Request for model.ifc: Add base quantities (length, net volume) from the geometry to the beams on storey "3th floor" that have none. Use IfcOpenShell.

First a look at what the model holds.

```python
import ifcopenshell
import ifcopenshell.util.element
import ifcopenshell.util.unit

model = ifcopenshell.open("model.ifc")
print(model.schema)
for unit_type in ("LENGTHUNIT", "AREAUNIT", "VOLUMEUNIT"):
    print(unit_type, ifcopenshell.util.unit.calculate_unit_scale(model, unit_type))
storey = next(s for s in model.by_type("IfcBuildingStorey") if s.Name == "3th floor")
beams = [e for e in ifcopenshell.util.element.get_decomposition(storey) if e.is_a("IfcBeam")]
for e in sorted(beams, key=lambda e: e.id()):
    print(e.id(), e.is_a(), e.Name, list(ifcopenshell.util.element.get_psets(e, qtos_only=True)), sep=" | ")
```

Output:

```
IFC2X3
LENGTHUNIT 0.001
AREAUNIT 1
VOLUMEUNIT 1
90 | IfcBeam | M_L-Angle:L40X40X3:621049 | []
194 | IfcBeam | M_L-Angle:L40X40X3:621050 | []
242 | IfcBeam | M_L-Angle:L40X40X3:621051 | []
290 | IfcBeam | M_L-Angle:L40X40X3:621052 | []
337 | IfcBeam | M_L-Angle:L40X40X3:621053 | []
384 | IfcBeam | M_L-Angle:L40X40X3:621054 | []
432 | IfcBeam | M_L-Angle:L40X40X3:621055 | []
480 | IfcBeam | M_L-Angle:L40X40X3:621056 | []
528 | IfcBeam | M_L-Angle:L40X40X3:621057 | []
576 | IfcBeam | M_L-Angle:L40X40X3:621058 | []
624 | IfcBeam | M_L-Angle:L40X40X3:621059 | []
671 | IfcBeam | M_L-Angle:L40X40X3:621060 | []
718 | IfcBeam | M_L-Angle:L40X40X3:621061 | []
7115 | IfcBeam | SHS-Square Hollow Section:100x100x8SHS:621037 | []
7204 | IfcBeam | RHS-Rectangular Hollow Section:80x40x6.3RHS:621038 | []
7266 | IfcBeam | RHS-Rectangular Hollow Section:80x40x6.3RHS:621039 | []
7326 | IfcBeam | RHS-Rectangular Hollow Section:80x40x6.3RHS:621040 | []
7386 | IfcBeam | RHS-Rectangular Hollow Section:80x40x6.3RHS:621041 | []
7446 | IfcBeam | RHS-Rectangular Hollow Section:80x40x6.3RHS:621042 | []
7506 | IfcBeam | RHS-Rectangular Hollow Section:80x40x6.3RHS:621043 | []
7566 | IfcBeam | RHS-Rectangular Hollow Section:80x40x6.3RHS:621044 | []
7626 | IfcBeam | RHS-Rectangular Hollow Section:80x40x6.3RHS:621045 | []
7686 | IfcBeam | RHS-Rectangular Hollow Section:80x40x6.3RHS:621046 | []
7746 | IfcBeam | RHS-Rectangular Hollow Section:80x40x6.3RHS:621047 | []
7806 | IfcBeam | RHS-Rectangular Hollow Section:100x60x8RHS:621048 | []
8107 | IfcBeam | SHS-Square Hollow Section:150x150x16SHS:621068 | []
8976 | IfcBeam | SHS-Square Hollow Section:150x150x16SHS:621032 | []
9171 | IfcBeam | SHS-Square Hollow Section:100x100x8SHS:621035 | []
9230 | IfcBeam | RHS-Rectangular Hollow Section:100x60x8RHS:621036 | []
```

```python
import ifcopenshell
import ifcopenshell.api.pset
import ifcopenshell.geom
import ifcopenshell.util.element
import ifcopenshell.util.shape
import ifcopenshell.util.unit

model = ifcopenshell.open("model.ifc")
unit_scale = ifcopenshell.util.unit.calculate_unit_scale(model)
volume_scale = ifcopenshell.util.unit.calculate_unit_scale(model, "VOLUMEUNIT")
settings = ifcopenshell.geom.settings()

storey = next(s for s in model.by_type("IfcBuildingStorey") if s.Name == "3th floor")
beams = [e for e in ifcopenshell.util.element.get_decomposition(storey) if e.is_a("IfcBeam")]

for e in sorted(beams, key=lambda e: e.id()):
    if ifcopenshell.util.element.get_psets(e, qtos_only=True, should_inherit=False):
        continue
    # Geometry comes back in metres, in the element's own axes.
    shape = ifcopenshell.geom.create_shape(settings, e)
    values = {
        "Length": ifcopenshell.util.shape.get_max_xyz(shape.geometry) / unit_scale,
        "NetVolume": ifcopenshell.util.shape.get_volume(shape.geometry) / volume_scale,
    }
    qto = ifcopenshell.api.pset.add_qto(model, product=e, name="BaseQuantities")
    ifcopenshell.api.pset.edit_qto(model, qto=qto, properties=values)
    print(e.id(), {k: round(v, 3) for k, v in values.items()})

model.write("model_updated.ifc")
```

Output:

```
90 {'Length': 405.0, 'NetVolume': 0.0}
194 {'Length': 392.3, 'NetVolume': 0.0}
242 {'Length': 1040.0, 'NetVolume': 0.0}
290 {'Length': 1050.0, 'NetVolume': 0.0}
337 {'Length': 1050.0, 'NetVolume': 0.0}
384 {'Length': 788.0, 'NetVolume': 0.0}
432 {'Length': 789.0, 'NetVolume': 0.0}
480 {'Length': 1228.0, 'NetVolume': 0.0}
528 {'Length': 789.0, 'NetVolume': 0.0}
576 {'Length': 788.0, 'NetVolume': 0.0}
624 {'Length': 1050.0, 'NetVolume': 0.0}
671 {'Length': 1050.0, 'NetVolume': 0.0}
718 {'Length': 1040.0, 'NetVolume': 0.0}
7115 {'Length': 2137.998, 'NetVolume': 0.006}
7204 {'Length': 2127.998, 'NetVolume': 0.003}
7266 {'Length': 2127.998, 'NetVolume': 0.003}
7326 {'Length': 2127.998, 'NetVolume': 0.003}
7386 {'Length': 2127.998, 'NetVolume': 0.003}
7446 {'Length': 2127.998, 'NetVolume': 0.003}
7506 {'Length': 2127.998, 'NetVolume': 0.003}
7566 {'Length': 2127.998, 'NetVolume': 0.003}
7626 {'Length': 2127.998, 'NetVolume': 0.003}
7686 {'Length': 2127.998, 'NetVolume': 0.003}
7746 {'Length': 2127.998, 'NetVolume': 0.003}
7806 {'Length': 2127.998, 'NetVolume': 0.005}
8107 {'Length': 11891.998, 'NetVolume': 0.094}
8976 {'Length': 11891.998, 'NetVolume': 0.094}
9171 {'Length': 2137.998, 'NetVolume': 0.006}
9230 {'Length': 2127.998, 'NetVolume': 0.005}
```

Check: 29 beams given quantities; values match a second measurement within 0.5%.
